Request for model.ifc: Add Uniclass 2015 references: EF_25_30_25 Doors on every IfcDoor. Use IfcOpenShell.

First a look at what the model holds.

```python
import ifcopenshell

model = ifcopenshell.open("model.ifc")
print(model.schema)
print("classifications:", [c.Name for c in model.by_type("IfcClassification")])
for ifc_class in ("IfcDoor", "IfcRoof", "IfcStair", "IfcWall", "IfcWindow"):
    print(ifc_class, len(model.by_type(ifc_class)))
```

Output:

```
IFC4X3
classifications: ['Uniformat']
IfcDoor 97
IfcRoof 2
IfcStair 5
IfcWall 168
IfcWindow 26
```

```python
import ifcopenshell
import ifcopenshell.api.classification

model = ifcopenshell.open("model.ifc")

system = ifcopenshell.api.classification.add_classification(model, classification="Uniclass 2015")

codes = {
    "IfcDoor": ("EF_25_30_25", "Doors"),
}
for ifc_class, (code, name) in codes.items():
    products = model.by_type(ifc_class)
    ifcopenshell.api.classification.add_reference(
        model, products=products, classification=system, identification=code, name=name
    )
    print(code, len(products))

model.write("model_edited.ifc")
```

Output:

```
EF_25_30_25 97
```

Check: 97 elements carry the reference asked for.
